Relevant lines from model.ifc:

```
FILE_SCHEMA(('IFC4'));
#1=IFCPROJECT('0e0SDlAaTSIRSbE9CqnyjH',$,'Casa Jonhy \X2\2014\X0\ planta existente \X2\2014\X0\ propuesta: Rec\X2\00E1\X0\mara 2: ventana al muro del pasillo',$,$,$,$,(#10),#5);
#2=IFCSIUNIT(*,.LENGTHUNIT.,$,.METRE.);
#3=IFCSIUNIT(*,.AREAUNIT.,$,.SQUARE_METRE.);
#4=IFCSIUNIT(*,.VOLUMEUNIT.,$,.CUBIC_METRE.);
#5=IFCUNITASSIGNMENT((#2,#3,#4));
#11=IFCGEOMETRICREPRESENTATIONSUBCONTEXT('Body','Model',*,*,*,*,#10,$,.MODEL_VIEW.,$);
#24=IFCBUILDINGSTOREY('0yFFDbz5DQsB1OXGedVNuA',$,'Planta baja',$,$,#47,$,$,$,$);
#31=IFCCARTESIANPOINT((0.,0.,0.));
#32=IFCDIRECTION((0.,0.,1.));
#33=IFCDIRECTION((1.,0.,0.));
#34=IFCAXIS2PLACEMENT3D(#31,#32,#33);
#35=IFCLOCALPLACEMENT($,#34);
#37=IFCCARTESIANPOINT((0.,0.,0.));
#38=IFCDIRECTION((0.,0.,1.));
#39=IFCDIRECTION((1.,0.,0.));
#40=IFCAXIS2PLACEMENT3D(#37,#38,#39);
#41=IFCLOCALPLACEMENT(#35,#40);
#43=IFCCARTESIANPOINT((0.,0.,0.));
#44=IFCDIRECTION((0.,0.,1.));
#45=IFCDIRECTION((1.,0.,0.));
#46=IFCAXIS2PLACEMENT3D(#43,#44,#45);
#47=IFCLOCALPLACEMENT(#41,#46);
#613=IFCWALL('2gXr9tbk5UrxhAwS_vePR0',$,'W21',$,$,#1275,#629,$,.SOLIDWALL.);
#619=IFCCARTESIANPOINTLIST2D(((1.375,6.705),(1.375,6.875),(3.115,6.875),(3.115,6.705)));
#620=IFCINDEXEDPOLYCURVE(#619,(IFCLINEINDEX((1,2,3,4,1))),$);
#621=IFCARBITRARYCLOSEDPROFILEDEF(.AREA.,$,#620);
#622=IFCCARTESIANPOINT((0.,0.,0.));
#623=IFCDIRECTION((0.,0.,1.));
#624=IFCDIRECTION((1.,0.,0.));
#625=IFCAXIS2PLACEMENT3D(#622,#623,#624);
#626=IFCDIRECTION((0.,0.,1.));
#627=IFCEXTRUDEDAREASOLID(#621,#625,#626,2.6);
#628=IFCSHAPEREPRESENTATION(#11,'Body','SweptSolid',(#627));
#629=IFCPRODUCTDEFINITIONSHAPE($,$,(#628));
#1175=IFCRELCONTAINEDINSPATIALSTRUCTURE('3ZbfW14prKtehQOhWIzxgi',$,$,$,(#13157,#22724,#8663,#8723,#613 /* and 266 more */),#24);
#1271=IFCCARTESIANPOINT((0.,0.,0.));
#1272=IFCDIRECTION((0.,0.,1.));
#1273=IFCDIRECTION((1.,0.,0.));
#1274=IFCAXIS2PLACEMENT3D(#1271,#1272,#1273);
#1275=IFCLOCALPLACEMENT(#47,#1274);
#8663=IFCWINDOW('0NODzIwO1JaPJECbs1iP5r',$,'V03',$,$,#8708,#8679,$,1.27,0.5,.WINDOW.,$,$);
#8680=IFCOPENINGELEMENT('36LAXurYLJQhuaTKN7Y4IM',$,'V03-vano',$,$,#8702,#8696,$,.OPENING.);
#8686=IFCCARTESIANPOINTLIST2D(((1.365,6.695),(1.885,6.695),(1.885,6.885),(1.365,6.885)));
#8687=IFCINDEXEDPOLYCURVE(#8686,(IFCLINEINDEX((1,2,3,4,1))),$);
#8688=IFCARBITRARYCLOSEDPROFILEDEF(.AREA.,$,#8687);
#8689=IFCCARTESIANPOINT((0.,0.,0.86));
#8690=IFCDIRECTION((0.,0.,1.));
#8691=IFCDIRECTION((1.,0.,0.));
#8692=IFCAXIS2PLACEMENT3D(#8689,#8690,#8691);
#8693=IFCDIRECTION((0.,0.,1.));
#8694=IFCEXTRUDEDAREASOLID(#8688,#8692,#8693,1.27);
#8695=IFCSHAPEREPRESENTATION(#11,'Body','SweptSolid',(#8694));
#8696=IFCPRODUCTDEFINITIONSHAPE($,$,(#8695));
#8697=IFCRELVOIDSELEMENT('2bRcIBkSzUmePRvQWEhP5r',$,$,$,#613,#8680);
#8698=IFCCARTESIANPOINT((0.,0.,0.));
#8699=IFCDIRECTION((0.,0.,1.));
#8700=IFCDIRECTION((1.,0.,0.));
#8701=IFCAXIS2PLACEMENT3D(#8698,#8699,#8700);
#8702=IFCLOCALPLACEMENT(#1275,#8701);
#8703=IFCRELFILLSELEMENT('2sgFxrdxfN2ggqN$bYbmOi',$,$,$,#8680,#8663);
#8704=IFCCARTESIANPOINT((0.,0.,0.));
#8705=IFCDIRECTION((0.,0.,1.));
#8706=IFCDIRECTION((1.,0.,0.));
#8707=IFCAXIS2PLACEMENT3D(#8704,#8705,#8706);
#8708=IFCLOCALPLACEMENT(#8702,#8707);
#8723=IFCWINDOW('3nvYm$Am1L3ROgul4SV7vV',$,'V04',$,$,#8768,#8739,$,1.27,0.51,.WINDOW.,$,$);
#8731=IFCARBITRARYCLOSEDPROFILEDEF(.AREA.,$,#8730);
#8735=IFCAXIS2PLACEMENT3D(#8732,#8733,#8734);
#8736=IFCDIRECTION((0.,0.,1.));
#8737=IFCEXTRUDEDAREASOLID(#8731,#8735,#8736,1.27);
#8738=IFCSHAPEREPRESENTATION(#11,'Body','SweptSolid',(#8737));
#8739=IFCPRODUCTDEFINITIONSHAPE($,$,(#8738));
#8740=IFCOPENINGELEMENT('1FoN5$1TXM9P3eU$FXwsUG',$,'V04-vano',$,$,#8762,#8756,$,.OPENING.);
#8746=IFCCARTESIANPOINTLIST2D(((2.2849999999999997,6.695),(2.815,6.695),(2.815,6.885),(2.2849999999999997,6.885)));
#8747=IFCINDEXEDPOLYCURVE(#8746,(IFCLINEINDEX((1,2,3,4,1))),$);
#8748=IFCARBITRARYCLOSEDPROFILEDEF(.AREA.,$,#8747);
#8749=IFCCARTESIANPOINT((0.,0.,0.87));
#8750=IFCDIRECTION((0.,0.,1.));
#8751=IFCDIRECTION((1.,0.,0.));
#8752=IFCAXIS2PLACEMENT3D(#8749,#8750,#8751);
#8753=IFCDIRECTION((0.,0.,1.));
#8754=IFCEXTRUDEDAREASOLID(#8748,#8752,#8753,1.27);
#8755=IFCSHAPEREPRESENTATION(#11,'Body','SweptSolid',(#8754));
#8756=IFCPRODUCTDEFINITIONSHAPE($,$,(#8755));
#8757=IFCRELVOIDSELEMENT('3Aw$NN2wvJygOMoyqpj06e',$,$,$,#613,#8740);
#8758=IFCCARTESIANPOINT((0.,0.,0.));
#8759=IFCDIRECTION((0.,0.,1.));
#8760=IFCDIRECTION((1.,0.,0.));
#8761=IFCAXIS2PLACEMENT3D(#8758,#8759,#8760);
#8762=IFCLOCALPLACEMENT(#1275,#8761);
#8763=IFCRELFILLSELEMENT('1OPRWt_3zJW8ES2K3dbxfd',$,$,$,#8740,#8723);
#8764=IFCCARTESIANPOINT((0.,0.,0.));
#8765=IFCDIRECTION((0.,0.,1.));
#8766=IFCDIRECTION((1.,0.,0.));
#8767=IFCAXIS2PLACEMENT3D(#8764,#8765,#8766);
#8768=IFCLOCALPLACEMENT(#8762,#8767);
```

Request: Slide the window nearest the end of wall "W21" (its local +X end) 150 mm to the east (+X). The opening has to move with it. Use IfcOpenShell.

```python
import ifcopenshell
import ifcopenshell.api.geometry
import ifcopenshell.util.placement

model = ifcopenshell.open("model.ifc")

window = model.by_guid("3nvYm$Am1L3ROgul4SV7vV")
opening = window.FillsVoids[0].RelatingOpeningElement
wall = opening.VoidsElements[0].RelatingBuildingElement

wall_matrix = ifcopenshell.util.placement.get_local_placement(wall.ObjectPlacement)
shift = wall_matrix[:3, 0] * 0.15
before = ifcopenshell.util.placement.get_local_placement(window.ObjectPlacement)[:3, 3].copy()

# The window is placed relative to its opening, so it follows when the opening moves.
matrix = ifcopenshell.util.placement.get_local_placement(opening.ObjectPlacement)
matrix[:3, 3] += shift
ifcopenshell.api.geometry.edit_object_placement(
    model, product=opening, matrix=matrix, is_si=False, should_transform_children=True
)

after = ifcopenshell.util.placement.get_local_placement(window.ObjectPlacement)[:3, 3]
print("window moved by", (after - before).round(3) + 0.0)

model.write("model-out.ifc")
```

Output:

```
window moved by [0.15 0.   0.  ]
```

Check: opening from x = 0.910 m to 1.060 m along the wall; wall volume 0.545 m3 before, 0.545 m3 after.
